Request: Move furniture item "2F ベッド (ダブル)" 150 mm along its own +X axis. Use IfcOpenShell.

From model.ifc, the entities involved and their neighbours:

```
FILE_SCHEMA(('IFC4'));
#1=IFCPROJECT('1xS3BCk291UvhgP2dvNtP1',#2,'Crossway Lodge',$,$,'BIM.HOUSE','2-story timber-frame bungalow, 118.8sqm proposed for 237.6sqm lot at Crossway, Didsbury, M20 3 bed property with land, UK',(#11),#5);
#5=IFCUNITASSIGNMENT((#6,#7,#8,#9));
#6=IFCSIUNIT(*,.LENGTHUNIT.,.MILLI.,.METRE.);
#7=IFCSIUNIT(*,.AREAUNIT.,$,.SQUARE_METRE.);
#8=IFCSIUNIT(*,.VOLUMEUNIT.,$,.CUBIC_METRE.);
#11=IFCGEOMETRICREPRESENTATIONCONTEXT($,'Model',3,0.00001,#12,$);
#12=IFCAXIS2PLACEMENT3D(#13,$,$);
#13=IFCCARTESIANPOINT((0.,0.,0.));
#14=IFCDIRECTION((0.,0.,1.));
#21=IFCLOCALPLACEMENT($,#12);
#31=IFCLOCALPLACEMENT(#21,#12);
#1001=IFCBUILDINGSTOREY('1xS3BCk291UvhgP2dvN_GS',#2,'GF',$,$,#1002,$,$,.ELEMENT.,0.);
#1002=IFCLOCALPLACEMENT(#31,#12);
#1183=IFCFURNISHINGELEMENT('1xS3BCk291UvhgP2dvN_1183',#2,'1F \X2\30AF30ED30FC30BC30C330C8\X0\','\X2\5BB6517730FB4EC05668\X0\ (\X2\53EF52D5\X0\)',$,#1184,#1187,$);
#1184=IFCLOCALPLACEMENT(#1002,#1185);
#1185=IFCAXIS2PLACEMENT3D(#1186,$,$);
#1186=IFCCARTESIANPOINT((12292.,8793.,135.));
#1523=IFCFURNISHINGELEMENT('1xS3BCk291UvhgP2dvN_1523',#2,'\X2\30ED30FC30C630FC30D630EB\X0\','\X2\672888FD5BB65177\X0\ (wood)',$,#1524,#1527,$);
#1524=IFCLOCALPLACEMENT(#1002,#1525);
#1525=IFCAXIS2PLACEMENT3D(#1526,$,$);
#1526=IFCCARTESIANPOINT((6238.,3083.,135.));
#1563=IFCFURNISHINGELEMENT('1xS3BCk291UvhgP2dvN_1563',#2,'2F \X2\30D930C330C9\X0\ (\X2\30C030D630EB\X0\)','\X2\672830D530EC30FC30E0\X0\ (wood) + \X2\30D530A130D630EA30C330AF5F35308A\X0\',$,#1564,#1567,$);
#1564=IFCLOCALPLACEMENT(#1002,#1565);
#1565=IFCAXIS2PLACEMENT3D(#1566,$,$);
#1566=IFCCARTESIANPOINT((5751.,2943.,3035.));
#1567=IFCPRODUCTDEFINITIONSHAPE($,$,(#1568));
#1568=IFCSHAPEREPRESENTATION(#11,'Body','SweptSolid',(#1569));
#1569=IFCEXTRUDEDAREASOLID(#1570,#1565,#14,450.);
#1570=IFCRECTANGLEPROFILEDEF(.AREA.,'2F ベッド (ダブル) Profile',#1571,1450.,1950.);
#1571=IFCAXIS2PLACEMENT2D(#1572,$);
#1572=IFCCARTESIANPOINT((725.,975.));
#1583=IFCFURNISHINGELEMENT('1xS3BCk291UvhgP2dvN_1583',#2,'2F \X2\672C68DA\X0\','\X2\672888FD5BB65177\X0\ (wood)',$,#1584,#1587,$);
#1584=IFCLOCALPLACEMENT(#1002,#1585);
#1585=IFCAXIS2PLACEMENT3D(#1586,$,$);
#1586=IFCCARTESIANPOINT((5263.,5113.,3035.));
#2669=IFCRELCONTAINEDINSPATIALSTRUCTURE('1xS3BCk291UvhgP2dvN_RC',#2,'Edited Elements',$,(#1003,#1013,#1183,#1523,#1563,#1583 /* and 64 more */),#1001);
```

```python
import ifcopenshell
import ifcopenshell.api.geometry
import ifcopenshell.util.placement
import ifcopenshell.util.unit

model = ifcopenshell.open("model.ifc")
unit_scale = ifcopenshell.util.unit.calculate_unit_scale(model)

item = model.by_id(1563)
matrix = ifcopenshell.util.placement.get_local_placement(item.ObjectPlacement)
matrix[:3, 3] += matrix[:3, 0] * 0.15 / unit_scale
ifcopenshell.api.geometry.edit_object_placement(model, product=item, matrix=matrix, is_si=False)

print(ifcopenshell.util.placement.get_local_placement(item.ObjectPlacement).round(3) + 0.0)

model.write("model_rev.ifc")
```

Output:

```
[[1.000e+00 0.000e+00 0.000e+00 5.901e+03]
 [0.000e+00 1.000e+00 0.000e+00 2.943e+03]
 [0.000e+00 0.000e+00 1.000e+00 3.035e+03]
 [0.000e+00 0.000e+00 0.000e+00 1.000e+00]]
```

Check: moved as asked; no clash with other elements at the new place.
